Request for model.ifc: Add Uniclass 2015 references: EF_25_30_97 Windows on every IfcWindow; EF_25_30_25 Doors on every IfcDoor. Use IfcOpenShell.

First a look at what the model holds.

```python
import ifcopenshell

model = ifcopenshell.open("model.ifc")
print(model.schema)
print("classifications:", [c.Name for c in model.by_type("IfcClassification")])
for ifc_class in ("IfcDoor", "IfcRoof", "IfcStair", "IfcWall", "IfcWindow"):
    print(ifc_class, len(model.by_type(ifc_class)))
```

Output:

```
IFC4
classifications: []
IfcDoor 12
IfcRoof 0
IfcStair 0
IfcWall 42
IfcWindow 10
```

```python
import ifcopenshell
import ifcopenshell.api.classification

model = ifcopenshell.open("model.ifc")

system = ifcopenshell.api.classification.add_classification(model, classification="Uniclass 2015")

codes = {
    "IfcWindow": ("EF_25_30_97", "Windows"),
    "IfcDoor": ("EF_25_30_25", "Doors"),
}
for ifc_class, (code, name) in codes.items():
    products = model.by_type(ifc_class)
    ifcopenshell.api.classification.add_reference(
        model, products=products, classification=system, identification=code, name=name
    )
    print(code, len(products))

model.write("model-out.ifc")
```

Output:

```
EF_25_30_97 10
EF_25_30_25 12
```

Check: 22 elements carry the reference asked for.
